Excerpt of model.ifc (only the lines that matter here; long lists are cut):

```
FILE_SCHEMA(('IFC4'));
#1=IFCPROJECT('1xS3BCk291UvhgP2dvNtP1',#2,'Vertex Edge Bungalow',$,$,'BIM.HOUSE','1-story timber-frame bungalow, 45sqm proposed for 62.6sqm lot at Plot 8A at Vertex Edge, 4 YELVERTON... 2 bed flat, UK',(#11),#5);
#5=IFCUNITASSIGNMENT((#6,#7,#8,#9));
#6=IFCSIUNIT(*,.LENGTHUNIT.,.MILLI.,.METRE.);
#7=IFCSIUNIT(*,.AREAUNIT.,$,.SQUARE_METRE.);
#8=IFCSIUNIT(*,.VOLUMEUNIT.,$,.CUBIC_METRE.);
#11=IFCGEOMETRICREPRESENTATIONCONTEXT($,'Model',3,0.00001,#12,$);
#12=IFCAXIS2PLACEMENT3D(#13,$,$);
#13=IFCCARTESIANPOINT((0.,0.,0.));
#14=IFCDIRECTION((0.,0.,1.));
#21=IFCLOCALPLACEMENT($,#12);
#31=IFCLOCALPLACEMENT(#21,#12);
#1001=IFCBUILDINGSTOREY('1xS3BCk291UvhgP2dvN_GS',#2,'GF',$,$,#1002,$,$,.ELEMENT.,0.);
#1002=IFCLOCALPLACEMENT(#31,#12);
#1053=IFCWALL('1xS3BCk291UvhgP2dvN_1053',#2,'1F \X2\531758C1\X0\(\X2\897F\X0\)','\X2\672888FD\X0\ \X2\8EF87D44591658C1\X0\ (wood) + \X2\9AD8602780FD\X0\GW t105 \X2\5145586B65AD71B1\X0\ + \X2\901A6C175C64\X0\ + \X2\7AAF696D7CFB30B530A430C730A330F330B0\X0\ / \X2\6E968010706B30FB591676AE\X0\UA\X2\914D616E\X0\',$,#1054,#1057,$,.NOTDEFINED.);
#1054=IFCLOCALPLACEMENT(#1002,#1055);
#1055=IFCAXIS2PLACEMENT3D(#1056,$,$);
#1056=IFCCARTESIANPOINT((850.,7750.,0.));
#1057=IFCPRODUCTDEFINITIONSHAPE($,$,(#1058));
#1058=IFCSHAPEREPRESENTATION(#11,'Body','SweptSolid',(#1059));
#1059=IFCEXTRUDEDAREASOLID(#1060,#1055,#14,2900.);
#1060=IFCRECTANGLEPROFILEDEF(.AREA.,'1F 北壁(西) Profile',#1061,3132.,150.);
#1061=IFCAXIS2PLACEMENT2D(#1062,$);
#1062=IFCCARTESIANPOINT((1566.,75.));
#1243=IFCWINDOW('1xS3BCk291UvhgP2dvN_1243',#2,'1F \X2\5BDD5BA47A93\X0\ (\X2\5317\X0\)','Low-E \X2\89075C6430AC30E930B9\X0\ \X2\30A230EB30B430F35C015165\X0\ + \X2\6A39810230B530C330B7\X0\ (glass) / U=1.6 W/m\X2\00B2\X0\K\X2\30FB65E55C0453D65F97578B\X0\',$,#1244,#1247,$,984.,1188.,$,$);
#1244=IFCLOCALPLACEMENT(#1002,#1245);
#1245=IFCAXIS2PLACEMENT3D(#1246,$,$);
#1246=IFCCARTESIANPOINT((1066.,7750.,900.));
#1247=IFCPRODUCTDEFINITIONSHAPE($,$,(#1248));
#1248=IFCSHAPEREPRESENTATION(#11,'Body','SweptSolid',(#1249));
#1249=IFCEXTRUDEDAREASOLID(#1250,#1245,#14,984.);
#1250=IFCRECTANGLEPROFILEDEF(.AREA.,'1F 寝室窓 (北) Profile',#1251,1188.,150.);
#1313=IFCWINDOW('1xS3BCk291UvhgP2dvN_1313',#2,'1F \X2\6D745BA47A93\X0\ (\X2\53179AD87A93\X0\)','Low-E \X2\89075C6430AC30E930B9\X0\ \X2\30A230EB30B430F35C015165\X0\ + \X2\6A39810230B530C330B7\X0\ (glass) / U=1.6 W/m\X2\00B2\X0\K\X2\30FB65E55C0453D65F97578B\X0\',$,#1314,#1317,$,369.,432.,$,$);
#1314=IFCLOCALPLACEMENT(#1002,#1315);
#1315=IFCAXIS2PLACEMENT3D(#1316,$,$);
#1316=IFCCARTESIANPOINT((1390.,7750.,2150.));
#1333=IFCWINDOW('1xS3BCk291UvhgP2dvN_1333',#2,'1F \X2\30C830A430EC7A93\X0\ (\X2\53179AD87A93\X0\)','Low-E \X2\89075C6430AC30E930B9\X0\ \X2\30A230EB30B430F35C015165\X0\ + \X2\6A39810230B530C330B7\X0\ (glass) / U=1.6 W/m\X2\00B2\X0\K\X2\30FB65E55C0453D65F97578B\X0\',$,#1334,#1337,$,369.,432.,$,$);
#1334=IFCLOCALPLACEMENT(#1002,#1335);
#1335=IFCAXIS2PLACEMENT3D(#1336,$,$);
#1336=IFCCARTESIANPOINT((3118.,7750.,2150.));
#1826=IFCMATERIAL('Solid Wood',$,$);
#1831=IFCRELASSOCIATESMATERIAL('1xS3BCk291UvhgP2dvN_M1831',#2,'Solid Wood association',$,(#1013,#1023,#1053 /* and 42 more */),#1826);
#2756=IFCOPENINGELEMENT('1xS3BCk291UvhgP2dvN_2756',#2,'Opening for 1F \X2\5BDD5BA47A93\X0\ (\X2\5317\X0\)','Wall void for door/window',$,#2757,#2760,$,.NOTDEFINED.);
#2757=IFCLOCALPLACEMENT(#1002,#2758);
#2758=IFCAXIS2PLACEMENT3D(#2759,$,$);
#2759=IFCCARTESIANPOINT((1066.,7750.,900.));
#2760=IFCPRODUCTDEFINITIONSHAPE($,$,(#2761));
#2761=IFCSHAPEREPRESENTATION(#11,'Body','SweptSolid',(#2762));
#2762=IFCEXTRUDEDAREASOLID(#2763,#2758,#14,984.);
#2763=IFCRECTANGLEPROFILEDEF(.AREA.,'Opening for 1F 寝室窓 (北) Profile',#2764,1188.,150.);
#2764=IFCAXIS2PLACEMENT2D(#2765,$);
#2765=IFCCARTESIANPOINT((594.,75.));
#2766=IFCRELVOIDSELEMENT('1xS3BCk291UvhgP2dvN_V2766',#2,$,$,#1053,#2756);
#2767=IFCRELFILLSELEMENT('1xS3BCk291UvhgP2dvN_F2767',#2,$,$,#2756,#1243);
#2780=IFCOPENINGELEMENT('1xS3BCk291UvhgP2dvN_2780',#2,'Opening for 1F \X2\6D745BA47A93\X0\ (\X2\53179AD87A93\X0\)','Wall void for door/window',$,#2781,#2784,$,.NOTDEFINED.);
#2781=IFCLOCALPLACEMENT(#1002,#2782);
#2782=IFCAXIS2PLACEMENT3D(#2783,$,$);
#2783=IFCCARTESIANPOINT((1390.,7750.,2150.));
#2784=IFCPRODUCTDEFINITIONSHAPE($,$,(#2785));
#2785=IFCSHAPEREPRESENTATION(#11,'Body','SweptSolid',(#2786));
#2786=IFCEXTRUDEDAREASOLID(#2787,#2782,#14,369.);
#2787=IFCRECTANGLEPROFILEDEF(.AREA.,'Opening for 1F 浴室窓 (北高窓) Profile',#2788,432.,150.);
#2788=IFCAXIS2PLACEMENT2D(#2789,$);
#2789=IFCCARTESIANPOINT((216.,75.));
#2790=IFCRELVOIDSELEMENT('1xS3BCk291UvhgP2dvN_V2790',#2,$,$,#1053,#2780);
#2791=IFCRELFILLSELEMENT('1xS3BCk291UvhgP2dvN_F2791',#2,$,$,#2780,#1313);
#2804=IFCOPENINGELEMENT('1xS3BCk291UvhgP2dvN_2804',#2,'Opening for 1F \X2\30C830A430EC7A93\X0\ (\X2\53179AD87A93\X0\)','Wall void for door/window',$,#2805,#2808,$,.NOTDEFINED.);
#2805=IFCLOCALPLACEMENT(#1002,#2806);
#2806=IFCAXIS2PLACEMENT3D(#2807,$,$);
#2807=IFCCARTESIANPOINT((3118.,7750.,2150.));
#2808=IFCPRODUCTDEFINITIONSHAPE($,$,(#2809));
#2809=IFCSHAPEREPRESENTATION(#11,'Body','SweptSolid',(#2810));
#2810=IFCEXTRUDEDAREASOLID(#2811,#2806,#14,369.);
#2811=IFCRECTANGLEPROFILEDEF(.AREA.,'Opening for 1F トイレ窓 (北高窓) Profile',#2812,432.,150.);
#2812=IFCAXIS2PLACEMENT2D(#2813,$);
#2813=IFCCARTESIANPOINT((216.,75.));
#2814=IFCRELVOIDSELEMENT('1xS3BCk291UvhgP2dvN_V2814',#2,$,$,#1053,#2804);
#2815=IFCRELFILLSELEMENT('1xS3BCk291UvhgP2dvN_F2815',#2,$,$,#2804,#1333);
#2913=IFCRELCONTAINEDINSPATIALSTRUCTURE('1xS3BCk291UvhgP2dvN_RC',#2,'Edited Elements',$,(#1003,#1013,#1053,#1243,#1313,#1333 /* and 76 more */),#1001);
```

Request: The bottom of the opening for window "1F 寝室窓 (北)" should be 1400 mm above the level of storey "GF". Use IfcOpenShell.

```python
import numpy as np
import ifcopenshell
import ifcopenshell.api.geometry
import ifcopenshell.geom
import ifcopenshell.util.element
import ifcopenshell.util.placement
import ifcopenshell.util.shape
import ifcopenshell.util.unit

model = ifcopenshell.open("model.ifc")
unit_scale = ifcopenshell.util.unit.calculate_unit_scale(model)

window = model.by_id(1243)
opening = window.FillsVoids[0].RelatingOpeningElement
storey = ifcopenshell.util.element.get_container(window, ifc_class="IfcBuildingStorey")
level = ifcopenshell.util.placement.get_local_placement(storey.ObjectPlacement)[2, 3]

# The opening's origin need not be at the sill, so measure its lowest point.
shape = ifcopenshell.geom.create_shape(ifcopenshell.geom.settings(), opening)
bottom = ifcopenshell.util.shape.get_shape_bottom_elevation(shape, shape.geometry) / unit_scale
dz = level + 1400.0 - bottom

shift = np.array([0.0, 0.0, dz])
# The window is not placed relative to its opening, so move both.
for product in (opening, window):
    matrix = ifcopenshell.util.placement.get_local_placement(product.ObjectPlacement)
    matrix[:3, 3] += shift
    ifcopenshell.api.geometry.edit_object_placement(model, product=product, matrix=matrix, is_si=False)

print(f"moved by {dz * unit_scale:+.3f} m")

model.write("model_v2.ifc")
```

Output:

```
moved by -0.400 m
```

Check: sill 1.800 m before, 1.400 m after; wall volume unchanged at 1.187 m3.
